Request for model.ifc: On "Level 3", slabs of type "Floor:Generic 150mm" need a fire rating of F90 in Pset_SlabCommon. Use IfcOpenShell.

First a look at what the model holds.

```python
import ifcopenshell
import ifcopenshell.util.element

model = ifcopenshell.open("model.ifc")
print(model.schema)
storey = next(s for s in model.by_type("IfcBuildingStorey") if s.Name == "Level 3")
slabs = [e for e in ifcopenshell.util.element.get_decomposition(storey) if e.is_a("IfcSlab")]
seen = {}
for e in slabs:
    element_type = ifcopenshell.util.element.get_type(e)
    key = (element_type.Name if element_type != e and element_type else None, ifcopenshell.util.element.get_pset(e, "Pset_SlabCommon", "FireRating"))
    seen[key] = seen.get(key, 0) + 1
for (name, value), count in sorted(seen.items(), key=str):
    print(count, "x", name, "|", value)
```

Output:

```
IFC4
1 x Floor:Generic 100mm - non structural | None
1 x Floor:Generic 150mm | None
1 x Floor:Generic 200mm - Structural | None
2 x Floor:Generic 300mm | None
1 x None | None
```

```python
import ifcopenshell
import ifcopenshell.api.pset
import ifcopenshell.util.element

model = ifcopenshell.open("model.ifc")

storey = next(s for s in model.by_type("IfcBuildingStorey") if s.Name == "Level 3")
slabs = [e for e in ifcopenshell.util.element.get_decomposition(storey) if e.is_a("IfcSlab")]

count = 0
for e in slabs:
    element_type = ifcopenshell.util.element.get_type(e)
    if element_type in (None, e) or element_type.Name != "Floor:Generic 150mm":
        continue
    # add_pset returns the element's existing set when there is one.
    pset = ifcopenshell.api.pset.add_pset(model, product=e, name="Pset_SlabCommon")
    ifcopenshell.api.pset.edit_pset(model, pset=pset, properties={"FireRating": "F90"})
    count += 1

print(count, "slabs updated")

model.write("model_edited.ifc")
```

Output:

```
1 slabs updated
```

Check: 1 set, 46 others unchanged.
